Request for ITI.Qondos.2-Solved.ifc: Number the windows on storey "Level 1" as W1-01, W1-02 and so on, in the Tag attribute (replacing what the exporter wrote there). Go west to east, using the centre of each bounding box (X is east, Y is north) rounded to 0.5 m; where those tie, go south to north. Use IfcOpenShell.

First a look at what the model holds.

```python
import ifcopenshell
import ifcopenshell.util.element
import ifcopenshell.util.placement

model = ifcopenshell.open("ITI.Qondos.2-Solved.ifc")
print(model.schema)
storey = next(s for s in model.by_type("IfcBuildingStorey") if s.Name == "Level 1")
windows = [e for e in ifcopenshell.util.element.get_decomposition(storey) if e.is_a("IfcWindow")]
for e in sorted(windows, key=lambda e: e.id()):
    origin = ifcopenshell.util.placement.get_local_placement(e.ObjectPlacement)[:3, 3]
    print(e.id(), e.Tag, e.Name, origin.round(2) + 0.0, sep=" | ")
```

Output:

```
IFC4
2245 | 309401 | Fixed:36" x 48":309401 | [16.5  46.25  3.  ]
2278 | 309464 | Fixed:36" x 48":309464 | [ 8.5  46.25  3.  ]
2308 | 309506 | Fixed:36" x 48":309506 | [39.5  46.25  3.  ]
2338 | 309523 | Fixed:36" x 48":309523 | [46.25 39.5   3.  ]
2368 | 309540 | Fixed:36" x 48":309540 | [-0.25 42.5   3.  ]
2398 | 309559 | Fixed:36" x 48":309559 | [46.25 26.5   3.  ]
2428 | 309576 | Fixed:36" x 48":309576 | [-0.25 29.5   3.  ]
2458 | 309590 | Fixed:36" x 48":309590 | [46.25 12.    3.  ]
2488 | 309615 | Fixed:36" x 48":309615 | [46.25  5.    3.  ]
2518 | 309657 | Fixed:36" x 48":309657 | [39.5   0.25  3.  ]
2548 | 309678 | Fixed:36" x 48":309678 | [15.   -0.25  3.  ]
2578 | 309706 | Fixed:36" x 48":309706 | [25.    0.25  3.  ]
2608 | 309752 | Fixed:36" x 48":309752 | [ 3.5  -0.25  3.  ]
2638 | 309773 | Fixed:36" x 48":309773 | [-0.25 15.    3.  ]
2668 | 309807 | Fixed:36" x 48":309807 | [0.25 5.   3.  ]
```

```python
import ifcopenshell
import ifcopenshell.geom
import ifcopenshell.util.element
import ifcopenshell.util.shape

model = ifcopenshell.open("ITI.Qondos.2-Solved.ifc")
settings = ifcopenshell.geom.settings()
settings.set("use-world-coords", True)


def centre(element):
    shape = ifcopenshell.geom.create_shape(settings, element)
    return ifcopenshell.util.shape.get_bbox_centroid(shape.geometry)


storey = next(s for s in model.by_type("IfcBuildingStorey") if s.Name == "Level 1")
windows = [e for e in ifcopenshell.util.element.get_decomposition(storey) if e.is_a("IfcWindow")]

# Insertion points can sit at a corner or the storey origin, so sort by the geometry (in metres).
centres = {e: centre(e) for e in windows}
windows.sort(key=lambda e: (round(centres[e][0] / 0.5), centres[e][1]))

for i, e in enumerate(windows, start=1):
    number = f"W1-{i:02d}"
    e.Tag = number
    print(e.id(), number)

model.write("ITI.Qondos.2-Solved_v2.ifc")
```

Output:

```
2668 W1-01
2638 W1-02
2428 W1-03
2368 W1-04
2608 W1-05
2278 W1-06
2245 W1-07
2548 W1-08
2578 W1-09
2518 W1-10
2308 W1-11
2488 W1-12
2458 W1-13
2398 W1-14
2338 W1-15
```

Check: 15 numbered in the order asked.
